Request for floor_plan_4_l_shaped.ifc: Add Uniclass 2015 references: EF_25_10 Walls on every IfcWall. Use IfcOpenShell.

First a look at what the model holds.

```python
import ifcopenshell

model = ifcopenshell.open("floor_plan_4_l_shaped.ifc")
print(model.schema)
print("classifications:", [c.Name for c in model.by_type("IfcClassification")])
for ifc_class in ("IfcDoor", "IfcRoof", "IfcStair", "IfcWall", "IfcWindow"):
    print(ifc_class, len(model.by_type(ifc_class)))
```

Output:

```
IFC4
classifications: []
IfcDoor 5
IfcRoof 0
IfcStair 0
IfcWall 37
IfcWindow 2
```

```python
import ifcopenshell
import ifcopenshell.api.classification

model = ifcopenshell.open("floor_plan_4_l_shaped.ifc")

system = ifcopenshell.api.classification.add_classification(model, classification="Uniclass 2015")

codes = {
    "IfcWall": ("EF_25_10", "Walls"),
}
for ifc_class, (code, name) in codes.items():
    products = model.by_type(ifc_class)
    ifcopenshell.api.classification.add_reference(
        model, products=products, classification=system, identification=code, name=name
    )
    print(code, len(products))

model.write("floor_plan_4_l_shaped_updated.ifc")
```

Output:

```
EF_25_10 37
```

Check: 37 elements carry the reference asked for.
